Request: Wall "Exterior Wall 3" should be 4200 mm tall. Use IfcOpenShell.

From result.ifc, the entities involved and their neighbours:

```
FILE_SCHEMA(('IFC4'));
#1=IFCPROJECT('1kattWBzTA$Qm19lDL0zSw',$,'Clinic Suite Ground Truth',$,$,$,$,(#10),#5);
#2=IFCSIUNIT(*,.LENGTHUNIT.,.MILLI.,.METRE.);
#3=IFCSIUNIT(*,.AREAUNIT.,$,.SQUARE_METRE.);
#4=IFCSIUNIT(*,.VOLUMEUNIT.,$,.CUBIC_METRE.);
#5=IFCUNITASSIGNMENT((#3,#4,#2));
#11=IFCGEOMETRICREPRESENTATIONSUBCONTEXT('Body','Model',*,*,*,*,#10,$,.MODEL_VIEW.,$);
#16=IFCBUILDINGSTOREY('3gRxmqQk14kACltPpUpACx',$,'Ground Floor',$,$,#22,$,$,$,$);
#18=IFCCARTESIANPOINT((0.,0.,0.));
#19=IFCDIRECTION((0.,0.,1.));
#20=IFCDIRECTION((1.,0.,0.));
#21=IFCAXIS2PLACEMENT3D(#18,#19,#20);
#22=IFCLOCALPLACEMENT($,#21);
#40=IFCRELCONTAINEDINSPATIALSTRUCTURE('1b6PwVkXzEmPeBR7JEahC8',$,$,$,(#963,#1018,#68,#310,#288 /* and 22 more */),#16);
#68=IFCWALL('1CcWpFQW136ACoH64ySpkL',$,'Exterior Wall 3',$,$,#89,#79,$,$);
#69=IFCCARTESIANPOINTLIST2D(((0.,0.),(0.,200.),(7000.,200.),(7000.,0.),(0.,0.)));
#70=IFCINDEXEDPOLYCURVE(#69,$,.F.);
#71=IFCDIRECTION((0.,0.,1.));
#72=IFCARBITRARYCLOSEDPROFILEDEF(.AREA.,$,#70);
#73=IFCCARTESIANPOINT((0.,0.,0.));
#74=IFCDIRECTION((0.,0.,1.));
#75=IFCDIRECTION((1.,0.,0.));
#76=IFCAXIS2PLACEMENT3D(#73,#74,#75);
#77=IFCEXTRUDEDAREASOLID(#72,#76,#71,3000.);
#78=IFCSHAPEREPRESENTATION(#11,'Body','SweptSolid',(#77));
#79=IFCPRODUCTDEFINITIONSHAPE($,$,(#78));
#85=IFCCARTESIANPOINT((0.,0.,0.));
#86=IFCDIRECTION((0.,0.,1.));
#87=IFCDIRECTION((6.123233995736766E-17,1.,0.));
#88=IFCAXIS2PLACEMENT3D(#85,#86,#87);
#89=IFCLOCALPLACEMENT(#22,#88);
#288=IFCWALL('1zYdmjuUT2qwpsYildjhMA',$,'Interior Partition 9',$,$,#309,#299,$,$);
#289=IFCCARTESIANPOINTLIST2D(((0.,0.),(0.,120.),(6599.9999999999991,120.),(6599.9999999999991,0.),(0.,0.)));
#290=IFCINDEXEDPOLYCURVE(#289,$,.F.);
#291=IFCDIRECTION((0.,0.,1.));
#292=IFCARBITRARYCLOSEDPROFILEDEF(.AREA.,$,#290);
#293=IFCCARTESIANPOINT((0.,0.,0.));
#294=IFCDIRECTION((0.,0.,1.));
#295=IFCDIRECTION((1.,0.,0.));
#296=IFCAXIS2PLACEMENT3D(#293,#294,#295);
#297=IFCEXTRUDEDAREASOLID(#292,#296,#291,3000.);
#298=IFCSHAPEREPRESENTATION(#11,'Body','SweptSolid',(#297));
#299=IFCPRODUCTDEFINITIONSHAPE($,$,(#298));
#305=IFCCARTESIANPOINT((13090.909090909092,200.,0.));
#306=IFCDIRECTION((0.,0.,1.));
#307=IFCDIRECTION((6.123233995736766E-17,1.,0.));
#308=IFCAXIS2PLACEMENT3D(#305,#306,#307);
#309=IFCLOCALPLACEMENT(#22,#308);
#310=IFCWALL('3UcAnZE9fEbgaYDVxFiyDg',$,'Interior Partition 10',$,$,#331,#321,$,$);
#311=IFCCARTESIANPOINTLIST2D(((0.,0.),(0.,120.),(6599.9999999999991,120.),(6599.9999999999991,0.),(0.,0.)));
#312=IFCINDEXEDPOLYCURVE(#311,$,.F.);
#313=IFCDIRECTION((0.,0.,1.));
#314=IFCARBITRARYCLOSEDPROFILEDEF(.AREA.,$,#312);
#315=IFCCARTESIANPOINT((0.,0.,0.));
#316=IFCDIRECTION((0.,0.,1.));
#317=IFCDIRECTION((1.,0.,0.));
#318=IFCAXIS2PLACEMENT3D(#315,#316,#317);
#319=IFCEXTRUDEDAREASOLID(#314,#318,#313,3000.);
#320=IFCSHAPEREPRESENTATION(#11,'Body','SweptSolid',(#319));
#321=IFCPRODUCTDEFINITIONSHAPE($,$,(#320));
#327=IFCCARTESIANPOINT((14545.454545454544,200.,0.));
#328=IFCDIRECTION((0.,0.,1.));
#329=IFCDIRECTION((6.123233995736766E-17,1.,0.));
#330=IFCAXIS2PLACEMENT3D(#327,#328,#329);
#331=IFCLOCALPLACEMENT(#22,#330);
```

```python
import ifcopenshell
import ifcopenshell.geom
import ifcopenshell.util.representation
import ifcopenshell.util.shape

model = ifcopenshell.open("result.ifc")
settings = ifcopenshell.geom.settings()


def volume(element):
    """Net volume in cubic metres, openings subtracted."""
    shape = ifcopenshell.geom.create_shape(settings, element)
    return ifcopenshell.util.shape.get_volume(shape.geometry)


wall = model.by_guid("1CcWpFQW136ACoH64ySpkL")
before = volume(wall)

body = ifcopenshell.util.representation.get_representation(wall, "Model", "Body")
solid = body.Items[0]
old_height = solid.Depth
solid.Depth = 4200.0
after = volume(wall)

print(f"height {old_height:g} -> {solid.Depth:g}, volume {before:.3f} -> {after:.3f} m3")

model.write("result_updated.ifc")
```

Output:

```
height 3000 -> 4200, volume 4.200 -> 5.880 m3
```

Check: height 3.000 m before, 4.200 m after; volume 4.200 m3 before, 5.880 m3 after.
